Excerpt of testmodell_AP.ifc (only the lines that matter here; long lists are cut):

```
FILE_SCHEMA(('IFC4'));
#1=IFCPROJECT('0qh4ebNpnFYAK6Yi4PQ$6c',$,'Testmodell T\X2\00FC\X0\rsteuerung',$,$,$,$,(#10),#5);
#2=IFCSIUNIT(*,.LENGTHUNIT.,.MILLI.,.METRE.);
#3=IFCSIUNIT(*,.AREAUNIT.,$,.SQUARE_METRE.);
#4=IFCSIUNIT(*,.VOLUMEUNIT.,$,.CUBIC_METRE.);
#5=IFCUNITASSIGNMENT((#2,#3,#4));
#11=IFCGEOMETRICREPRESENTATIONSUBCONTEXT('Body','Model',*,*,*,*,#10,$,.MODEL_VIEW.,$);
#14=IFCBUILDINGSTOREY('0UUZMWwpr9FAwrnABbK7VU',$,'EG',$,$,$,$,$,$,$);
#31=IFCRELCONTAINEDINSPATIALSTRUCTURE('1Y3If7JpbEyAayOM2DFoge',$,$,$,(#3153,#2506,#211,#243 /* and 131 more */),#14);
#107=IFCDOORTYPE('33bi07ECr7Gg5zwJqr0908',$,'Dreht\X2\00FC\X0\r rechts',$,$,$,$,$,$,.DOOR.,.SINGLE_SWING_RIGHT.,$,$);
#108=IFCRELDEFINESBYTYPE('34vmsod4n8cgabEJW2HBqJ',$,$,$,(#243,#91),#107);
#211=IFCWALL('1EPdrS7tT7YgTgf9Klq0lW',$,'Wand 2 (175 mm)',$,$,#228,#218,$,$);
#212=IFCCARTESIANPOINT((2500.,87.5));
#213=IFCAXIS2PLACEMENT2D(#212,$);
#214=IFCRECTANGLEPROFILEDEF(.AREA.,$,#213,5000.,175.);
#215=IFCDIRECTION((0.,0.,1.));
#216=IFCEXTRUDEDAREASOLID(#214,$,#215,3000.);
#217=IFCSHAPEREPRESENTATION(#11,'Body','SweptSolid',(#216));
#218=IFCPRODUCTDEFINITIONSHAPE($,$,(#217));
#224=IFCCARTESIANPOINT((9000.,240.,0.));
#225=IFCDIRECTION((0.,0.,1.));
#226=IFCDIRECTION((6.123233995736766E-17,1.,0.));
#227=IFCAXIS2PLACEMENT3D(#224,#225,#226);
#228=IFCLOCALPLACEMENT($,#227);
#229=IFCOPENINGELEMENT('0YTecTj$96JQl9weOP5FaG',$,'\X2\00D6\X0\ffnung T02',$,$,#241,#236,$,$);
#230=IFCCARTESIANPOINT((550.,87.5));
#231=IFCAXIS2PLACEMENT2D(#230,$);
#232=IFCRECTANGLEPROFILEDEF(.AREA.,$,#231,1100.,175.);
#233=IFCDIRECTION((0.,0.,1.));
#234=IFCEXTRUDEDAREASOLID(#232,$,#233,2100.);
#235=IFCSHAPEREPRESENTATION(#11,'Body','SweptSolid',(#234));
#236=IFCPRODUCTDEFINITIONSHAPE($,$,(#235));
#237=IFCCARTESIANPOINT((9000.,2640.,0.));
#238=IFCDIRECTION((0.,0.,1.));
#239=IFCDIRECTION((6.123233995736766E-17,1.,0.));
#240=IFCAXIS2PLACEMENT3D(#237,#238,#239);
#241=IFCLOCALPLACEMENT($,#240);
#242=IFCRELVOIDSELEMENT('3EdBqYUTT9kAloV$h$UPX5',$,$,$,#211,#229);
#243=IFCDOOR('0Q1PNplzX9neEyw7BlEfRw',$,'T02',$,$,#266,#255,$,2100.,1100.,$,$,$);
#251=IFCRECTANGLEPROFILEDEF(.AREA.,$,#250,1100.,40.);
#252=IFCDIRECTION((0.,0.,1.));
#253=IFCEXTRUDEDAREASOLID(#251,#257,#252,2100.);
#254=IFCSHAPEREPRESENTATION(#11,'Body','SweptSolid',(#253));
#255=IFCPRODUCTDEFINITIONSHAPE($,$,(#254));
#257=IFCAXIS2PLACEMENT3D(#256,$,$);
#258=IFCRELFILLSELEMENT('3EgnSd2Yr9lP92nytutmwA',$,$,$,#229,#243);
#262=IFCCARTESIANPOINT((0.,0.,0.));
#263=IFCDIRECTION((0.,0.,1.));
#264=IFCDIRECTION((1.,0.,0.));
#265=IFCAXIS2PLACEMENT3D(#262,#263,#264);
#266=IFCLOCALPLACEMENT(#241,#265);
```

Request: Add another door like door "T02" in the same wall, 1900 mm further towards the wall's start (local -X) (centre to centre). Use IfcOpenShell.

```python
import ifcopenshell
import ifcopenshell.api.feature
import ifcopenshell.api.geometry
import ifcopenshell.api.root
import ifcopenshell.geom
import ifcopenshell.util.element
import ifcopenshell.util.placement
import ifcopenshell.util.shape

model = ifcopenshell.open("testmodell_AP.ifc")
settings = ifcopenshell.geom.settings()


def volume(element):
    """Net volume in cubic metres, openings subtracted."""
    shape = ifcopenshell.geom.create_shape(settings, element)
    return ifcopenshell.util.shape.get_volume(shape.geometry)


door = model.by_guid("0Q1PNplzX9neEyw7BlEfRw")
opening = door.FillsVoids[0].RelatingOpeningElement
wall = opening.VoidsElements[0].RelatingBuildingElement
before = volume(wall)
shift = ifcopenshell.util.placement.get_local_placement(wall.ObjectPlacement)[:3, 0] * -1900.0

# copy_class copies the void relationship, type, container and properties, but no geometry.
new_opening = ifcopenshell.api.root.copy_class(model, product=opening)
new_opening.Representation = ifcopenshell.util.element.copy_deep(
    model, opening.Representation, exclude=["IfcGeometricRepresentationContext", "IfcRepresentationMap"]
)
new_door = ifcopenshell.api.root.copy_class(model, product=door)
new_door.Representation = ifcopenshell.util.element.copy_deep(
    model, door.Representation, exclude=["IfcGeometricRepresentationContext", "IfcRepresentationMap"]
)
ifcopenshell.api.feature.add_filling(model, opening=new_opening, element=new_door)

for old, new in ((opening, new_opening), (door, new_door)):
    matrix = ifcopenshell.util.placement.get_local_placement(old.ObjectPlacement)
    matrix[:3, 3] += shift
    ifcopenshell.api.geometry.edit_object_placement(model, product=new, matrix=matrix, is_si=False)

after = volume(wall)

print(f"wall volume {before:.3f} -> {after:.3f} m3")

model.write("testmodell_AP_updated.ifc")
```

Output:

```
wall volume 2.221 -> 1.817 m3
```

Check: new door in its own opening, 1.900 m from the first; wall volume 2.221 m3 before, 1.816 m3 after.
